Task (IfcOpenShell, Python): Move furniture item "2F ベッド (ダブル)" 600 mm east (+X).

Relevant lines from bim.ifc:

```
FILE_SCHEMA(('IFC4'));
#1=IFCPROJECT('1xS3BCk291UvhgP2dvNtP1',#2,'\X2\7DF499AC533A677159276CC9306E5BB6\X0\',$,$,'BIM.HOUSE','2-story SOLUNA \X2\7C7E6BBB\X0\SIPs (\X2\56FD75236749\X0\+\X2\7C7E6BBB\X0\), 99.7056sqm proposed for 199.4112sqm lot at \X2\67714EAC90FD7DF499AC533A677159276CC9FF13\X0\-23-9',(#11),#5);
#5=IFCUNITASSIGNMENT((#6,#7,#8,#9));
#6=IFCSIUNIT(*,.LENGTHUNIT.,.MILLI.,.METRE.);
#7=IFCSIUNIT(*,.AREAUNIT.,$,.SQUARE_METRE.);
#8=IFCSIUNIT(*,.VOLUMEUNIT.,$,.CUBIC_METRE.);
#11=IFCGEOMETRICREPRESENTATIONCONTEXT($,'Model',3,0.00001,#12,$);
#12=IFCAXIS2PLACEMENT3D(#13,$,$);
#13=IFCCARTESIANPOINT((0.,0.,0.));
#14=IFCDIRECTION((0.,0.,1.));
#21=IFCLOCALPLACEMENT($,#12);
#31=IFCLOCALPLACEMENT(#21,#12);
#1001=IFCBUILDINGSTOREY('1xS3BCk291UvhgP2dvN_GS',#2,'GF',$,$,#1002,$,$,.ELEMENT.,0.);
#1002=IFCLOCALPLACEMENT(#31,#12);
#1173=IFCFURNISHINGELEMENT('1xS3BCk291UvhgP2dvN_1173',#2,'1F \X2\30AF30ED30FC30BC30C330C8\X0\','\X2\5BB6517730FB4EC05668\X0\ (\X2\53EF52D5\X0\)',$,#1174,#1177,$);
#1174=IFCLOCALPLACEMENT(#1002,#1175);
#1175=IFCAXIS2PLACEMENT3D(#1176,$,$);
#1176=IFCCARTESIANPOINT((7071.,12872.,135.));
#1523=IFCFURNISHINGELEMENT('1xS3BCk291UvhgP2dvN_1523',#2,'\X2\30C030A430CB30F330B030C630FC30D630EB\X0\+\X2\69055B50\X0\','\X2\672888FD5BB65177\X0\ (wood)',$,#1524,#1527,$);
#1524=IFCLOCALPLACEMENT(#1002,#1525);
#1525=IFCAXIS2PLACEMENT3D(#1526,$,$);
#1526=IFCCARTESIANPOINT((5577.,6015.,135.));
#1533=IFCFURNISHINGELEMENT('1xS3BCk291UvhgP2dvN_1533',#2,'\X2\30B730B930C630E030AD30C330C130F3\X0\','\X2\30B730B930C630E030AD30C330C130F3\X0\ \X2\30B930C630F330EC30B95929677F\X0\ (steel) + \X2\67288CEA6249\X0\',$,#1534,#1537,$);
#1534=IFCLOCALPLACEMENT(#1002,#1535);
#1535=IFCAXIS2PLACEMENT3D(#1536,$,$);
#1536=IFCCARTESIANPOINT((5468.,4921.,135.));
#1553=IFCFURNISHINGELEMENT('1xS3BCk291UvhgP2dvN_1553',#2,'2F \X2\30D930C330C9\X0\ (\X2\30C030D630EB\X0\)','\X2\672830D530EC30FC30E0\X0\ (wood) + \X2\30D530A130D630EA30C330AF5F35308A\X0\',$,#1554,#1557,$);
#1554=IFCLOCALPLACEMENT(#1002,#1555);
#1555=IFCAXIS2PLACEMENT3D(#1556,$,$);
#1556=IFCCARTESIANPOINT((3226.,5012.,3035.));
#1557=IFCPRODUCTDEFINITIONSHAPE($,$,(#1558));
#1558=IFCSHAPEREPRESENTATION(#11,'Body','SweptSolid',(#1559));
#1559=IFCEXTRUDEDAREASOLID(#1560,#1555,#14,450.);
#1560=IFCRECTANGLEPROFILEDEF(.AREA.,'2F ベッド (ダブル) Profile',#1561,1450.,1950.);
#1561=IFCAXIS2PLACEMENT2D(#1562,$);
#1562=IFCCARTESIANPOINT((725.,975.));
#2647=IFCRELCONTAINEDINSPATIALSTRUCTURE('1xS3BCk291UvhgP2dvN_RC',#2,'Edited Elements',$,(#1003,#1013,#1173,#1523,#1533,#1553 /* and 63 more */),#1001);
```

```python
import ifcopenshell
import ifcopenshell.api.geometry
import ifcopenshell.util.placement
import ifcopenshell.util.unit

model = ifcopenshell.open("bim.ifc")
unit_scale = ifcopenshell.util.unit.calculate_unit_scale(model)

item = model.by_guid("1xS3BCk291UvhgP2dvN_1553")
matrix = ifcopenshell.util.placement.get_local_placement(item.ObjectPlacement)
matrix[0, 3] += 0.6 / unit_scale
ifcopenshell.api.geometry.edit_object_placement(model, product=item, matrix=matrix, is_si=False)

print(ifcopenshell.util.placement.get_local_placement(item.ObjectPlacement).round(3) + 0.0)

model.write("bim_edited.ifc")
```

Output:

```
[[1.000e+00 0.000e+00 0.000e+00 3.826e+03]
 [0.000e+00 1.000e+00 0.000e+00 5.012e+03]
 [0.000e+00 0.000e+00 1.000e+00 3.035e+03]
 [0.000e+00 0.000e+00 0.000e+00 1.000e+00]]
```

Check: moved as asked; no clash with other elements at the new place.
